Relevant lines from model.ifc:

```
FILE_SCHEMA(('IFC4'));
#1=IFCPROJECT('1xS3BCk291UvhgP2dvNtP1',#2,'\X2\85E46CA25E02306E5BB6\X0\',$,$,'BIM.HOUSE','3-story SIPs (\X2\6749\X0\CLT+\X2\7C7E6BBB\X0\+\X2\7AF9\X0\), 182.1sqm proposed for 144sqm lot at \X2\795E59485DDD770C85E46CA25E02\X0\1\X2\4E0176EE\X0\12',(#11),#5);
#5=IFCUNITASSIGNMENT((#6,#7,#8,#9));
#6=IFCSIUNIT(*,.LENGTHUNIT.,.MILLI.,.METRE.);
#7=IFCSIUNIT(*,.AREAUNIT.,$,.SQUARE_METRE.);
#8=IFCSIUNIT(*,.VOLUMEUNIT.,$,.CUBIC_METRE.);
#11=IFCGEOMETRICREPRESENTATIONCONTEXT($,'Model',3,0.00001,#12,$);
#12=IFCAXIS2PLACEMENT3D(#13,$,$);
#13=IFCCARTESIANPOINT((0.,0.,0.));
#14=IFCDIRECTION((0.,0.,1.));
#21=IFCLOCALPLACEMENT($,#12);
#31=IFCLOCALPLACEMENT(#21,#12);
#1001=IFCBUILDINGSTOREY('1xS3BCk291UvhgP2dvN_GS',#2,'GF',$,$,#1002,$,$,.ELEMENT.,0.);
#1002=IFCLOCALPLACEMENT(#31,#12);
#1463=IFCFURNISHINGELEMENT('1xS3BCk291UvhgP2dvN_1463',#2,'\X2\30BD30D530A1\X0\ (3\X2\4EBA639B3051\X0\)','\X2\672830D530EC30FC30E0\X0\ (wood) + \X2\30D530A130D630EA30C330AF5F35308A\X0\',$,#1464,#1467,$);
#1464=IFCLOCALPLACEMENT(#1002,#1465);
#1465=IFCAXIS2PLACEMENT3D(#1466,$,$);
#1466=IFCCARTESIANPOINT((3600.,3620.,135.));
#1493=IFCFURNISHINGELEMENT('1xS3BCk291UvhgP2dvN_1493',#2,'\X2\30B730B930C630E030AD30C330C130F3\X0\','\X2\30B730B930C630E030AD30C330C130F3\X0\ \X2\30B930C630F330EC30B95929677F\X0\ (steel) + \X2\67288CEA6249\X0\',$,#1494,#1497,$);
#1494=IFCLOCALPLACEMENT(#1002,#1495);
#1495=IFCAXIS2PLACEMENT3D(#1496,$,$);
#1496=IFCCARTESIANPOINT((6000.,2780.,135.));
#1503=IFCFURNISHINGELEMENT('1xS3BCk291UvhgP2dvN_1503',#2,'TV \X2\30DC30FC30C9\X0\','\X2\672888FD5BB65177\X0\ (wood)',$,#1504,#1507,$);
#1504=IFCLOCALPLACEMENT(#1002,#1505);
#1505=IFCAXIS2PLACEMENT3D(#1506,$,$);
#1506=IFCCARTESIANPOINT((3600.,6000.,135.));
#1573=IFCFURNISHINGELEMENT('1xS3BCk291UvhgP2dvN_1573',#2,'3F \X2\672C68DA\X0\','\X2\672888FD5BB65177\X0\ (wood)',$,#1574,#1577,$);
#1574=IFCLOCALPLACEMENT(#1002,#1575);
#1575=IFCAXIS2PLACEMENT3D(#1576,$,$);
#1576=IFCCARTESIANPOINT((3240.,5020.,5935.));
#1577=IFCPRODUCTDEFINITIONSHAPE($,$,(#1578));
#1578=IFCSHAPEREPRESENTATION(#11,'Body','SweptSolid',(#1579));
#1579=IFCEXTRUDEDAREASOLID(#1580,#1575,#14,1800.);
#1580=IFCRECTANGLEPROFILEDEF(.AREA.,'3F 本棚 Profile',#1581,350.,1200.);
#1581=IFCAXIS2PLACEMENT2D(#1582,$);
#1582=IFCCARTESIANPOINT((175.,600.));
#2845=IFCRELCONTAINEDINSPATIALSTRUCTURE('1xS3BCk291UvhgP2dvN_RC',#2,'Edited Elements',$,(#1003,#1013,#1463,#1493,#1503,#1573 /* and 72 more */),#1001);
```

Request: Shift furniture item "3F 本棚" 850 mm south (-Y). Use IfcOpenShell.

```python
import ifcopenshell
import ifcopenshell.api.geometry
import ifcopenshell.util.placement
import ifcopenshell.util.unit

model = ifcopenshell.open("model.ifc")
unit_scale = ifcopenshell.util.unit.calculate_unit_scale(model)

item = model.by_guid("1xS3BCk291UvhgP2dvN_1573")
matrix = ifcopenshell.util.placement.get_local_placement(item.ObjectPlacement)
matrix[1, 3] -= 0.85 / unit_scale
ifcopenshell.api.geometry.edit_object_placement(model, product=item, matrix=matrix, is_si=False)

print(ifcopenshell.util.placement.get_local_placement(item.ObjectPlacement).round(3) + 0.0)

model.write("model_rev.ifc")
```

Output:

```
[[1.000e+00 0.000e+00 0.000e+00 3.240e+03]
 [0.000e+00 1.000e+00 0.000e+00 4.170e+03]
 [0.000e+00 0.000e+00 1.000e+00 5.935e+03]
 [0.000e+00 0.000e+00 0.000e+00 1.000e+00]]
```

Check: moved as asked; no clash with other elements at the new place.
